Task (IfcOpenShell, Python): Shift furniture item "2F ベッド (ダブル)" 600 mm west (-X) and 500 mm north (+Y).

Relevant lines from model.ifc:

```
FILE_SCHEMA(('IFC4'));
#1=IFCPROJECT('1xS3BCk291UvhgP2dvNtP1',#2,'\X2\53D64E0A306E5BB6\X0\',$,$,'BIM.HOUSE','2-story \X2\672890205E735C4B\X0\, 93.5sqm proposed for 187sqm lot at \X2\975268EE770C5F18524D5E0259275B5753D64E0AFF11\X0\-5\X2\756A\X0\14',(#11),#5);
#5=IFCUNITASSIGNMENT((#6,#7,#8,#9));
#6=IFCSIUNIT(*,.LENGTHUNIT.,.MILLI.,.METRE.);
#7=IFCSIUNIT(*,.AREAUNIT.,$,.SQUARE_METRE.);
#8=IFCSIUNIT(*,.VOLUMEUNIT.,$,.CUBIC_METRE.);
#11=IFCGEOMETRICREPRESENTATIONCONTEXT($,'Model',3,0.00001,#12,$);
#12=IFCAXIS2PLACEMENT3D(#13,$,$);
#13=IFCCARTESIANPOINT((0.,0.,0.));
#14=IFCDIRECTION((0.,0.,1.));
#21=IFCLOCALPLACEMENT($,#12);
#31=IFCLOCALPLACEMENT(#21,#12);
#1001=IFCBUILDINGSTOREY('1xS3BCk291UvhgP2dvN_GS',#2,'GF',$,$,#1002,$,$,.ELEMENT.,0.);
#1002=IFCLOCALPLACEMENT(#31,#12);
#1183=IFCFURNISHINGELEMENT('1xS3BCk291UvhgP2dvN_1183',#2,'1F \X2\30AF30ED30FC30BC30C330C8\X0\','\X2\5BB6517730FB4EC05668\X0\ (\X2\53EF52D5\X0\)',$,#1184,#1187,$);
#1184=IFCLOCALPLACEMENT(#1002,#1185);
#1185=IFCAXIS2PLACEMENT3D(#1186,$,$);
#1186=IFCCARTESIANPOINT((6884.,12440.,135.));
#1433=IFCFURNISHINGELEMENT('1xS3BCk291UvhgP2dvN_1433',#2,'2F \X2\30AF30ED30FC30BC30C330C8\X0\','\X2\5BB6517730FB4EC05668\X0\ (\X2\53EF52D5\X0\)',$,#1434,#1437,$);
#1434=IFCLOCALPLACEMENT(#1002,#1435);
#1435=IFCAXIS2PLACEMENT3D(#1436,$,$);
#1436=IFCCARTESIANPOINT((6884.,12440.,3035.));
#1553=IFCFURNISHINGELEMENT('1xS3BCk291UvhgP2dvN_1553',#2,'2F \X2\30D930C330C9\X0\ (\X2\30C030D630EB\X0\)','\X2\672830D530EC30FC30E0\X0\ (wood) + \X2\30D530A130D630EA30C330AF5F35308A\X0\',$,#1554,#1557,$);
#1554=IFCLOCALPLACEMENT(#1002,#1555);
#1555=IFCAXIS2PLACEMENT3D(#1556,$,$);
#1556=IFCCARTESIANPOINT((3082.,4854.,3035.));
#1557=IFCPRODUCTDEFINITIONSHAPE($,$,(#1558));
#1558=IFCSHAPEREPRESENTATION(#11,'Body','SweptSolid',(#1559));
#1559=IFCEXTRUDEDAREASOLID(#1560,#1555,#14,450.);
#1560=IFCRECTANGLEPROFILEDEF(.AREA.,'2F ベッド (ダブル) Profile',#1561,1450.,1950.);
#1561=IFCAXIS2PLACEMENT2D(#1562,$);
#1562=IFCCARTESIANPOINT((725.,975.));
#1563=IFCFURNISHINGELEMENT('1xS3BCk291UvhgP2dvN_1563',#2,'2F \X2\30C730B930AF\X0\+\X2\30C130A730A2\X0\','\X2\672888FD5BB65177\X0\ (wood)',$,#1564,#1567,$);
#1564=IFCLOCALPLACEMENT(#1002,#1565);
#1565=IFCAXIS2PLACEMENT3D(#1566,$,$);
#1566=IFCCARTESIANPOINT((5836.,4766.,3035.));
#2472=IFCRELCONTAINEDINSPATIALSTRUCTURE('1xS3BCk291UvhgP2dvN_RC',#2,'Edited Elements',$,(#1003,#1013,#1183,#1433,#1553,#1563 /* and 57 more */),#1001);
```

```python
import ifcopenshell
import ifcopenshell.api.geometry
import ifcopenshell.util.placement

model = ifcopenshell.open("model.ifc")

item = model.by_guid("1xS3BCk291UvhgP2dvN_1553")
matrix = ifcopenshell.util.placement.get_local_placement(item.ObjectPlacement)
matrix[0, 3] -= 600.0
matrix[1, 3] += 500.0
ifcopenshell.api.geometry.edit_object_placement(model, product=item, matrix=matrix, is_si=False)

print(ifcopenshell.util.placement.get_local_placement(item.ObjectPlacement).round(3) + 0.0)

model.write("model_edited.ifc")
```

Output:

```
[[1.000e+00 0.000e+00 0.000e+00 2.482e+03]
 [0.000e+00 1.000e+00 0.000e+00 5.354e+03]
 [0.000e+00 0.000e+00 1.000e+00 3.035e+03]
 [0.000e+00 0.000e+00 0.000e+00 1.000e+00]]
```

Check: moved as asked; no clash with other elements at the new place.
